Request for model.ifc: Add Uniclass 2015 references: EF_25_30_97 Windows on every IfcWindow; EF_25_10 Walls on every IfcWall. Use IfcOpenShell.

First a look at what the model holds.

```python
import ifcopenshell

model = ifcopenshell.open("model.ifc")
print(model.schema)
print("classifications:", [c.Name for c in model.by_type("IfcClassification")])
for ifc_class in ("IfcDoor", "IfcRoof", "IfcStair", "IfcWall", "IfcWindow"):
    print(ifc_class, len(model.by_type(ifc_class)))
```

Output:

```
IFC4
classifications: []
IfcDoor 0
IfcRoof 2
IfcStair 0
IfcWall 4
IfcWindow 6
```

```python
import ifcopenshell
import ifcopenshell.api.classification

model = ifcopenshell.open("model.ifc")

system = ifcopenshell.api.classification.add_classification(model, classification="Uniclass 2015")

codes = {
    "IfcWindow": ("EF_25_30_97", "Windows"),
    "IfcWall": ("EF_25_10", "Walls"),
}
for ifc_class, (code, name) in codes.items():
    products = model.by_type(ifc_class)
    ifcopenshell.api.classification.add_reference(
        model, products=products, classification=system, identification=code, name=name
    )
    print(code, len(products))

model.write("model_rev.ifc")
```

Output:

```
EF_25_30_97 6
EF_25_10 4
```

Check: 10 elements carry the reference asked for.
